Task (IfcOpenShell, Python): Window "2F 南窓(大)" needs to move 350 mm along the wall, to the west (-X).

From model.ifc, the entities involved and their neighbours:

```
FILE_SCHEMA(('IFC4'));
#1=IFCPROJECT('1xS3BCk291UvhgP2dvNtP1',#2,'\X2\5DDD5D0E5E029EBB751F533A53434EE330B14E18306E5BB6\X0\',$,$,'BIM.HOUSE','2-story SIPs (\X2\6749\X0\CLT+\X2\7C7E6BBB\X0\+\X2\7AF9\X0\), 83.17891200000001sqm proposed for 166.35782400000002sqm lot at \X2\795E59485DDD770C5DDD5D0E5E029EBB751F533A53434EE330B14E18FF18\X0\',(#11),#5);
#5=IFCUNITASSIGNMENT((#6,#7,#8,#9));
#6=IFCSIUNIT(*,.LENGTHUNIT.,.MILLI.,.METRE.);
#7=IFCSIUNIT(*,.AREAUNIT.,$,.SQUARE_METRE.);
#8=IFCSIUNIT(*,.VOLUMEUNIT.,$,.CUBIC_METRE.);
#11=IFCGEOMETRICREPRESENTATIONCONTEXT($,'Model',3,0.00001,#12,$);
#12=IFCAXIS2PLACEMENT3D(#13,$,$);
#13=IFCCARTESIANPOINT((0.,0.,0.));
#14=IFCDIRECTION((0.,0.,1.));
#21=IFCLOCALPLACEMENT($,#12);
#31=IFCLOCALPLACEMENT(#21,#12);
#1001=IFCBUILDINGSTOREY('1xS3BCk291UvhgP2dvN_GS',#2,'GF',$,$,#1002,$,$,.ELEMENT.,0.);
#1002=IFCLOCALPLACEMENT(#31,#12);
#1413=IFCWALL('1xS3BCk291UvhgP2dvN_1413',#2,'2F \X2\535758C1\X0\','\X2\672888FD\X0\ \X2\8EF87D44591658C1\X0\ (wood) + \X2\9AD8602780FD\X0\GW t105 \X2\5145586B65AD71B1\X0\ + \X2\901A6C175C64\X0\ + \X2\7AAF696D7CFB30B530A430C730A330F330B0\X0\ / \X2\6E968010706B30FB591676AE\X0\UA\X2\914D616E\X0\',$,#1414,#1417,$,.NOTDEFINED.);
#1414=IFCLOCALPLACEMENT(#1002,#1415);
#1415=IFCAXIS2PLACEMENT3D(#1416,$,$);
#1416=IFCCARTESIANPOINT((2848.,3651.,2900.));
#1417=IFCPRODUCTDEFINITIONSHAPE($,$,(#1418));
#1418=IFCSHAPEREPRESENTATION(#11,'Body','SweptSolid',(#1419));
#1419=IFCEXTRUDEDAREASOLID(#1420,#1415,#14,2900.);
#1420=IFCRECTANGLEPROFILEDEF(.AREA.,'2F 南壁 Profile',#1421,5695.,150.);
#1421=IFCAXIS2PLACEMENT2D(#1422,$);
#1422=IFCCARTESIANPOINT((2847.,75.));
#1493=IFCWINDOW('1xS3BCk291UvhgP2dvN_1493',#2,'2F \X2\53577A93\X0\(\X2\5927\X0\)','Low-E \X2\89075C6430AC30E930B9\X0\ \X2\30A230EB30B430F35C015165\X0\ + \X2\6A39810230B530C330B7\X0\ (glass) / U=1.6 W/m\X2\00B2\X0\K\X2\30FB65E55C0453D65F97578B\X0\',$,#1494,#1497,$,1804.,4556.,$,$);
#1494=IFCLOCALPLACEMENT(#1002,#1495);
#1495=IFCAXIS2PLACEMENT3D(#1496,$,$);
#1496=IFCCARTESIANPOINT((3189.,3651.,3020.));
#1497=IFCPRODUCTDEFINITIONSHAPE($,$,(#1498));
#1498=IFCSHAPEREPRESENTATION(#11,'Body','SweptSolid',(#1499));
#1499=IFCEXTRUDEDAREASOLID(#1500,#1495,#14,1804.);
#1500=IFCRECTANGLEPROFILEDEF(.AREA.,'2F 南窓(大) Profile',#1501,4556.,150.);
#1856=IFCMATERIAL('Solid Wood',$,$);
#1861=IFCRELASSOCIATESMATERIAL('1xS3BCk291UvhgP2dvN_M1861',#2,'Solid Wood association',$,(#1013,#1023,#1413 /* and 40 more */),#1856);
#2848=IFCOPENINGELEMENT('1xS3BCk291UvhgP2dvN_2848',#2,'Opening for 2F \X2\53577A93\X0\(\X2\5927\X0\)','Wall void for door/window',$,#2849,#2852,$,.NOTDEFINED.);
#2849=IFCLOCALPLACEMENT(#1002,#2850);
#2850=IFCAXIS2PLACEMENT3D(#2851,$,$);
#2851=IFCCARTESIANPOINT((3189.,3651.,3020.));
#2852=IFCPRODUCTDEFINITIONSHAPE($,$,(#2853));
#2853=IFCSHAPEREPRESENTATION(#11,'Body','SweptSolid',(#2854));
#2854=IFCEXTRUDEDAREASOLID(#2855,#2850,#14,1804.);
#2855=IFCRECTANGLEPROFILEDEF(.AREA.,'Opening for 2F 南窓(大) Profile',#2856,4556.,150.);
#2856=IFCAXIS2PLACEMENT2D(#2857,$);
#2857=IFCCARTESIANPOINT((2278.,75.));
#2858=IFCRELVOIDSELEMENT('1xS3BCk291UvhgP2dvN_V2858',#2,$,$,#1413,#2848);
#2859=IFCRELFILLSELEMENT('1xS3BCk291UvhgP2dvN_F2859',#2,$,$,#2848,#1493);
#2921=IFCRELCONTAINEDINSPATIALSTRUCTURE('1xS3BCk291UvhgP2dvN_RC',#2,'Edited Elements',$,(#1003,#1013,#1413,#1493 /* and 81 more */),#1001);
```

```python
import ifcopenshell
import ifcopenshell.api.geometry
import ifcopenshell.util.placement

model = ifcopenshell.open("model.ifc")

window = model.by_guid("1xS3BCk291UvhgP2dvN_1493")
opening = window.FillsVoids[0].RelatingOpeningElement
wall = opening.VoidsElements[0].RelatingBuildingElement

wall_matrix = ifcopenshell.util.placement.get_local_placement(wall.ObjectPlacement)
shift = wall_matrix[:3, 0] * -350.0
before = ifcopenshell.util.placement.get_local_placement(window.ObjectPlacement)[:3, 3].copy()

# The window is not placed relative to its opening, so move both.
for product in (opening, window):
    matrix = ifcopenshell.util.placement.get_local_placement(product.ObjectPlacement)
    matrix[:3, 3] += shift
    ifcopenshell.api.geometry.edit_object_placement(model, product=product, matrix=matrix, is_si=False)

after = ifcopenshell.util.placement.get_local_placement(window.ObjectPlacement)[:3, 3]
print("window moved by", (after - before).round(3) + 0.0)

model.write("model_edited.ifc")
```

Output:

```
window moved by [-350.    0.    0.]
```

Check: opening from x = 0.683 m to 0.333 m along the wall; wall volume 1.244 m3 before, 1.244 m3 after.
